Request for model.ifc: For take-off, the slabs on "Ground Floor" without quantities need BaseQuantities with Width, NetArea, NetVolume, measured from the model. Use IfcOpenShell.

First a look at what the model holds.

```python
import ifcopenshell
import ifcopenshell.util.element
import ifcopenshell.util.unit

model = ifcopenshell.open("model.ifc")
print(model.schema)
for unit_type in ("LENGTHUNIT", "AREAUNIT", "VOLUMEUNIT"):
    print(unit_type, ifcopenshell.util.unit.calculate_unit_scale(model, unit_type))
storey = next(s for s in model.by_type("IfcBuildingStorey") if s.Name == "Ground Floor")
slabs = [e for e in ifcopenshell.util.element.get_decomposition(storey) if e.is_a("IfcSlab")]
for e in sorted(slabs, key=lambda e: e.id()):
    print(e.id(), e.is_a(), e.Name, list(ifcopenshell.util.element.get_psets(e, qtos_only=True)), sep=" | ")
```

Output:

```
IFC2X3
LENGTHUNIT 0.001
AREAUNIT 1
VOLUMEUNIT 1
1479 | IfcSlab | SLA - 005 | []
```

```python
import ifcopenshell
import ifcopenshell.api.pset
import ifcopenshell.geom
import ifcopenshell.util.element
import ifcopenshell.util.shape
import ifcopenshell.util.unit

model = ifcopenshell.open("model.ifc")
unit_scale = ifcopenshell.util.unit.calculate_unit_scale(model)
area_scale = ifcopenshell.util.unit.calculate_unit_scale(model, "AREAUNIT")
volume_scale = ifcopenshell.util.unit.calculate_unit_scale(model, "VOLUMEUNIT")
settings = ifcopenshell.geom.settings()

storey = next(s for s in model.by_type("IfcBuildingStorey") if s.Name == "Ground Floor")
slabs = [e for e in ifcopenshell.util.element.get_decomposition(storey) if e.is_a("IfcSlab")]

for e in sorted(slabs, key=lambda e: e.id()):
    if ifcopenshell.util.element.get_psets(e, qtos_only=True, should_inherit=False):
        continue
    # Geometry comes back in metres, in the element's own axes.
    shape = ifcopenshell.geom.create_shape(settings, e)
    values = {
        "Width": ifcopenshell.util.shape.get_z(shape.geometry) / unit_scale,
        "NetArea": ifcopenshell.util.shape.get_footprint_area(shape.geometry) / area_scale,
        "NetVolume": ifcopenshell.util.shape.get_volume(shape.geometry) / volume_scale,
    }
    qto = ifcopenshell.api.pset.add_qto(model, product=e, name="BaseQuantities")
    ifcopenshell.api.pset.edit_qto(model, qto=qto, properties=values)
    print(e.id(), {k: round(v, 3) for k, v in values.items()})

model.write("model_v2.ifc")
```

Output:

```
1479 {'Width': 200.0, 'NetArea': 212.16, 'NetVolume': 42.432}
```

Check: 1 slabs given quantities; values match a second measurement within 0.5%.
